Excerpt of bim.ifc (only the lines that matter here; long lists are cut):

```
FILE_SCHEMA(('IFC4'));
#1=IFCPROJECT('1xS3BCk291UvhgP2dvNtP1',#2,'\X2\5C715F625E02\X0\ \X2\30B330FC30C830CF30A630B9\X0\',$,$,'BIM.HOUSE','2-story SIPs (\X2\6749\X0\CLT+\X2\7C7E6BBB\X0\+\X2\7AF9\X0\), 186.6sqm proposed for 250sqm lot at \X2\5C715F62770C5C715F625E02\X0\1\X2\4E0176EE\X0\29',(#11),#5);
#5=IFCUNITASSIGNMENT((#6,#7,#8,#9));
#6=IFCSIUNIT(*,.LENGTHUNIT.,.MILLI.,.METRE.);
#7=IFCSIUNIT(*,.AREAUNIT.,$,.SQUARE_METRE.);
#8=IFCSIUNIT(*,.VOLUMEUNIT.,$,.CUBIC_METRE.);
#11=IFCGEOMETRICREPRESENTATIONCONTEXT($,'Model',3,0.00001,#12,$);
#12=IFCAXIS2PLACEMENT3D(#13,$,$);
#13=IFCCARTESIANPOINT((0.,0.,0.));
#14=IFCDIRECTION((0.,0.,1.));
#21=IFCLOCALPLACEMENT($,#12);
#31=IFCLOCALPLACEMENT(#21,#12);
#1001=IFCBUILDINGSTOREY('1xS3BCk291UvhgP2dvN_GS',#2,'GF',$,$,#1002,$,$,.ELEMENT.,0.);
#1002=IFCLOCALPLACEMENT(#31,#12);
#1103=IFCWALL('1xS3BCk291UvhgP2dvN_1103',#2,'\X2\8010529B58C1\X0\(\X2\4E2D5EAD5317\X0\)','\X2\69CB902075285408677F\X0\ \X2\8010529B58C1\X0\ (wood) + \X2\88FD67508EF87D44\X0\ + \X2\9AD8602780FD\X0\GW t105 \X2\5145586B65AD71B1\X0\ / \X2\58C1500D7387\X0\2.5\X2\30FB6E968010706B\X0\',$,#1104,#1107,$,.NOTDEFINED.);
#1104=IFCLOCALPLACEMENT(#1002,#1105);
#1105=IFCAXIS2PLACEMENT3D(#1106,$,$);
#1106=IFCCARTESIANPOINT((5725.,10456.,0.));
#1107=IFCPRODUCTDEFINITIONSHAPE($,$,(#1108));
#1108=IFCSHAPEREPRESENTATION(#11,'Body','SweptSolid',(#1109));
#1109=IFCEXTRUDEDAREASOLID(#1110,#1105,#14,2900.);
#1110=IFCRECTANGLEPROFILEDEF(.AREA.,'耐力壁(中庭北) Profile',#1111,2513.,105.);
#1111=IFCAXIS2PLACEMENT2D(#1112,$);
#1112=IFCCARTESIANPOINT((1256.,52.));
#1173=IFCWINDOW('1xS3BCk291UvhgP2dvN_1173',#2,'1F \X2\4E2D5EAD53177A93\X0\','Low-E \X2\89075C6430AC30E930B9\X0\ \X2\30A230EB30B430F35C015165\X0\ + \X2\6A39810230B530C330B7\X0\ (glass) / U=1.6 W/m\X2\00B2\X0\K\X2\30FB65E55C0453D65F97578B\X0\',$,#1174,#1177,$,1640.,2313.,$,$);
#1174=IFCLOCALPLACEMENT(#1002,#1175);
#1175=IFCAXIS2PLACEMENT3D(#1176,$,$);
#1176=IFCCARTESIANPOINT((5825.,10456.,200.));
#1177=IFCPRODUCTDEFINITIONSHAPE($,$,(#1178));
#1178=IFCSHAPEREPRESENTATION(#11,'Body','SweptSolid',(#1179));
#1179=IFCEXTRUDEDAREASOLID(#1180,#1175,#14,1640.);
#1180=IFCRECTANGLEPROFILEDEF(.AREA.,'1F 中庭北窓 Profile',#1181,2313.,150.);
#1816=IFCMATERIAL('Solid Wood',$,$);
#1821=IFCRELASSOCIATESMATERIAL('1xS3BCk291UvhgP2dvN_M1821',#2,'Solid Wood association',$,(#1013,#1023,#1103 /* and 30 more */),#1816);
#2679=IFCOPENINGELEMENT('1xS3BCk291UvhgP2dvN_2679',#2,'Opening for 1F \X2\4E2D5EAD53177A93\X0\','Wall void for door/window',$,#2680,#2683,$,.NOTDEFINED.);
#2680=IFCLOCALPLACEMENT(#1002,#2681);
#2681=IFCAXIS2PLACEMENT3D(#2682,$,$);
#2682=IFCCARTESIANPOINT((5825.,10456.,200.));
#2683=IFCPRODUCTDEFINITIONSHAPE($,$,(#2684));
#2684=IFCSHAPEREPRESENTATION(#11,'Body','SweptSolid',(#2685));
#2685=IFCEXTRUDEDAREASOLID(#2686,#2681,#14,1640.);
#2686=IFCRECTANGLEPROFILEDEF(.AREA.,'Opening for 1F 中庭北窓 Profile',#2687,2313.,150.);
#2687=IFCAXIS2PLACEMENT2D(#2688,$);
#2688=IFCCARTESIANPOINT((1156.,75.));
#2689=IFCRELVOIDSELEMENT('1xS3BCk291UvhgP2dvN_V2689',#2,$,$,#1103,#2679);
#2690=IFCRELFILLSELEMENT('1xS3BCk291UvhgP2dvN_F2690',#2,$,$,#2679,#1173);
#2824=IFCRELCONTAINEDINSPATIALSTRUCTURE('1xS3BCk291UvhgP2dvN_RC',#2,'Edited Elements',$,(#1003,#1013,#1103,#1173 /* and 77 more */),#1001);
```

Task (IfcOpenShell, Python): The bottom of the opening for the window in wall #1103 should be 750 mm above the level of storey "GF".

```python
import numpy as np
import ifcopenshell
import ifcopenshell.api.geometry
import ifcopenshell.geom
import ifcopenshell.util.element
import ifcopenshell.util.placement
import ifcopenshell.util.shape
import ifcopenshell.util.unit

model = ifcopenshell.open("bim.ifc")
unit_scale = ifcopenshell.util.unit.calculate_unit_scale(model)

window = model.by_id(1173)
opening = window.FillsVoids[0].RelatingOpeningElement
storey = ifcopenshell.util.element.get_container(window, ifc_class="IfcBuildingStorey")
level = ifcopenshell.util.placement.get_local_placement(storey.ObjectPlacement)[2, 3]

# The opening's origin need not be at the sill, so measure its lowest point.
shape = ifcopenshell.geom.create_shape(ifcopenshell.geom.settings(), opening)
bottom = ifcopenshell.util.shape.get_shape_bottom_elevation(shape, shape.geometry) / unit_scale
dz = level + 0.75 / unit_scale - bottom

shift = np.array([0.0, 0.0, dz])
# The window is not placed relative to its opening, so move both.
for product in (opening, window):
    matrix = ifcopenshell.util.placement.get_local_placement(product.ObjectPlacement)
    matrix[:3, 3] += shift
    ifcopenshell.api.geometry.edit_object_placement(model, product=product, matrix=matrix, is_si=False)

print(f"moved by {dz * unit_scale:+.3f} m")

model.write("bim_updated.ifc")
```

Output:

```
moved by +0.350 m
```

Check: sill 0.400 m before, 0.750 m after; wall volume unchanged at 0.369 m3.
